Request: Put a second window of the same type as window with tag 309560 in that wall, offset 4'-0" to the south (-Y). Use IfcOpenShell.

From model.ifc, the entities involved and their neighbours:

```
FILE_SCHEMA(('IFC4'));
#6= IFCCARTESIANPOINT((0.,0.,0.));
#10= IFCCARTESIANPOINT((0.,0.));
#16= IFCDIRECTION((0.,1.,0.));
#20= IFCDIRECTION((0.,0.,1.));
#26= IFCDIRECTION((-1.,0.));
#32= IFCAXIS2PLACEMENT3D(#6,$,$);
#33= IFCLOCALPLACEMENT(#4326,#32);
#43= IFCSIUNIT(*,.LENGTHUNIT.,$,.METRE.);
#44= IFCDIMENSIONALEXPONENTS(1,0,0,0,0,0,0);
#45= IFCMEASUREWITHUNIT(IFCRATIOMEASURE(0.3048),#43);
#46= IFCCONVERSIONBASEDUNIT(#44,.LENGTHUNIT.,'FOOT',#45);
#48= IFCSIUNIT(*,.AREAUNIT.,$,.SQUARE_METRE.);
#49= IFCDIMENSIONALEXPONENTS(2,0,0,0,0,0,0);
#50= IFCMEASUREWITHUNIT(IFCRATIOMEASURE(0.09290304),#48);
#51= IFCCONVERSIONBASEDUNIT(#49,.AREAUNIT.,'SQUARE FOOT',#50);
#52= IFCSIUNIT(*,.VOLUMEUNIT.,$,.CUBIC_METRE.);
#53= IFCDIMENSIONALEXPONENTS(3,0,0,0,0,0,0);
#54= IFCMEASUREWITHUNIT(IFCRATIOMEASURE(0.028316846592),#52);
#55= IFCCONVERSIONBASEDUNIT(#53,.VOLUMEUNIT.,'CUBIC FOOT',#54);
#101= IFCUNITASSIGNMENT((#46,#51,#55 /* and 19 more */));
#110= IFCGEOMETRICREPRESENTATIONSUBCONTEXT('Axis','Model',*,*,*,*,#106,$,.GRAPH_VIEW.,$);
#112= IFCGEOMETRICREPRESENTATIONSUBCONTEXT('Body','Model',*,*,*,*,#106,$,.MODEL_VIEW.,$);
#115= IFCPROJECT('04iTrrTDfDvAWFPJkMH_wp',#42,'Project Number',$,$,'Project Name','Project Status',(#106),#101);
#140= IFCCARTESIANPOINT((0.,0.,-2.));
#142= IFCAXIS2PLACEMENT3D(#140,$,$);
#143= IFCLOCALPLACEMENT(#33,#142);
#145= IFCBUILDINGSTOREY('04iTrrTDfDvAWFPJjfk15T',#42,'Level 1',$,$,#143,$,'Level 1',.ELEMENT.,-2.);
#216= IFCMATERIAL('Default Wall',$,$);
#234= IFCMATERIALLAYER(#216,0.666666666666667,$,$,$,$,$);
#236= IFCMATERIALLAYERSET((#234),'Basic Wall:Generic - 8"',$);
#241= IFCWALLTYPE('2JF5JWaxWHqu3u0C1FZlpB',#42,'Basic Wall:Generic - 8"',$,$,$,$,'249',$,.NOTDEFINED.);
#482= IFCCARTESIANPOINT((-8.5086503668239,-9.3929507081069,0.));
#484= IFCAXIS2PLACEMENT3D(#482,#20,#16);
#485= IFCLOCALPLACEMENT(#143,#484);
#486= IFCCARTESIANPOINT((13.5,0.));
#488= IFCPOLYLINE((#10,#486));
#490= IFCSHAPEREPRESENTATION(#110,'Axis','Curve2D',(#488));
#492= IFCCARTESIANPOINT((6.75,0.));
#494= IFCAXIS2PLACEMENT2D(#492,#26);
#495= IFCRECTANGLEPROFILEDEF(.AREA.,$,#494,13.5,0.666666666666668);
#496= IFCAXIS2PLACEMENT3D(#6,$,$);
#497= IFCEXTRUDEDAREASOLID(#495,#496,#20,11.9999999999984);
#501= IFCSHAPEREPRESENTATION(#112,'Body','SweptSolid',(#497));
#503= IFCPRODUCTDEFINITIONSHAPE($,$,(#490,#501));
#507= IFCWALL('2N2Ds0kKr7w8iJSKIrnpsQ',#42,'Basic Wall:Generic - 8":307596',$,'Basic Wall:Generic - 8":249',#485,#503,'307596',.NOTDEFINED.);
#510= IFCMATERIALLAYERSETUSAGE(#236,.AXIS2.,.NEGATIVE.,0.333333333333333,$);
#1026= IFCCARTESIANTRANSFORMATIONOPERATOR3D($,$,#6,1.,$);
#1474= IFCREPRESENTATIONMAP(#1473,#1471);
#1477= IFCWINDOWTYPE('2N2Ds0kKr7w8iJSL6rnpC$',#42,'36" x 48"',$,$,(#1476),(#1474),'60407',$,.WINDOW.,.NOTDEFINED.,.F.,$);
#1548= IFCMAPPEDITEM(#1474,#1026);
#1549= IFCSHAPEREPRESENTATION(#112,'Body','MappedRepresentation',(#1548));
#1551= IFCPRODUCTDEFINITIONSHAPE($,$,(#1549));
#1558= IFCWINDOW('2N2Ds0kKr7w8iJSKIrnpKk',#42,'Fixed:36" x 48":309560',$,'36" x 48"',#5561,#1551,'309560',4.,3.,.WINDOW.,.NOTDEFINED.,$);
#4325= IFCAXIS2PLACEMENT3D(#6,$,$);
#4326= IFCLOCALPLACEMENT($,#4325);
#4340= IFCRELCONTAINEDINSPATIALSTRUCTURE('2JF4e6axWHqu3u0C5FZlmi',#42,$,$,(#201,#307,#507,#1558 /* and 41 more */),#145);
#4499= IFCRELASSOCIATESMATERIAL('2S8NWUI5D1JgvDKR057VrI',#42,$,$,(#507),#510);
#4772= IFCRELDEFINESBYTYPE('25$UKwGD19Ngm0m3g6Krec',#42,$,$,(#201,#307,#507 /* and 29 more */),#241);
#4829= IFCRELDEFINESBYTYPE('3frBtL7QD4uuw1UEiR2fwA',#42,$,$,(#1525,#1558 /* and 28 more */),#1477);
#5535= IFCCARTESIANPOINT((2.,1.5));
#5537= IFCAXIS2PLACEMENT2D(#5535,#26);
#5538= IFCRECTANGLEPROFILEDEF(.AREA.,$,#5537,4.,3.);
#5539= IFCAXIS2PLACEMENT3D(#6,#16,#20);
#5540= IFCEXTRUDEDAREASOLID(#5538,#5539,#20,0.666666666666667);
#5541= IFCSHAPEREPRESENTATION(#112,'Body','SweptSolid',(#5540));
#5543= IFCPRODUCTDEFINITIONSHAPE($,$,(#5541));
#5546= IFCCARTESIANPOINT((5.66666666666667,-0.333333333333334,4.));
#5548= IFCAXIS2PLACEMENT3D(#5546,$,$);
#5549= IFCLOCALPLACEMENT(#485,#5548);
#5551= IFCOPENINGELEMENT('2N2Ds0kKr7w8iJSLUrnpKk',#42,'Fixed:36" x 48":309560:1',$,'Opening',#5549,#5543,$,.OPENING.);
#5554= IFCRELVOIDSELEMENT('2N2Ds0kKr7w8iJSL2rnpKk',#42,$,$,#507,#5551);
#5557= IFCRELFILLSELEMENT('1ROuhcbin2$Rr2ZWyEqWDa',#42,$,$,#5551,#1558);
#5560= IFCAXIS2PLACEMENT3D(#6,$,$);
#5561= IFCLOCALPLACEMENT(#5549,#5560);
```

```python
import ifcopenshell
import ifcopenshell.api.feature
import ifcopenshell.api.geometry
import ifcopenshell.api.root
import ifcopenshell.geom
import ifcopenshell.util.element
import ifcopenshell.util.placement
import ifcopenshell.util.shape
import ifcopenshell.util.unit

model = ifcopenshell.open("model.ifc")
unit_scale = ifcopenshell.util.unit.calculate_unit_scale(model)
settings = ifcopenshell.geom.settings()


def volume(element):
    """Net volume in cubic metres, openings subtracted."""
    shape = ifcopenshell.geom.create_shape(settings, element)
    return ifcopenshell.util.shape.get_volume(shape.geometry)


def reuse_history(source, copy):
    """copy_class also copies each property set's owner history, people and application; keep the originals."""
    for rel in copy.IsDefinedBy:
        if rel.is_a("IfcRelDefinesByProperties") and (history := rel.RelatingPropertyDefinition.OwnerHistory):
            rel.RelatingPropertyDefinition.OwnerHistory = source.OwnerHistory
            ifcopenshell.util.element.remove_deep2(model, history)


window = model.by_id(1558)
opening = window.FillsVoids[0].RelatingOpeningElement
wall = opening.VoidsElements[0].RelatingBuildingElement
before = volume(wall)
shift = ifcopenshell.util.placement.get_local_placement(wall.ObjectPlacement)[:3, 0] * -48 * 0.0254 / unit_scale

# copy_class copies the void relationship, type, container and properties, but no geometry.
new_opening = ifcopenshell.api.root.copy_class(model, product=opening)
new_opening.Representation = ifcopenshell.util.element.copy_deep(
    model, opening.Representation, exclude=["IfcGeometricRepresentationContext", "IfcRepresentationMap"]
)
new_opening.Name = 'Fixed:36" x 48"'
new_window = ifcopenshell.api.root.copy_class(model, product=window)
new_window.Representation = ifcopenshell.util.element.copy_deep(
    model, window.Representation, exclude=["IfcGeometricRepresentationContext", "IfcRepresentationMap"]
)
new_window.Name = 'Fixed:36" x 48"'
new_window.Tag = None
reuse_history(window, new_window)
ifcopenshell.api.feature.add_filling(model, opening=new_opening, element=new_window)

for old, new in ((opening, new_opening), (window, new_window)):
    matrix = ifcopenshell.util.placement.get_local_placement(old.ObjectPlacement)
    matrix[:3, 3] += shift
    ifcopenshell.api.geometry.edit_object_placement(model, product=new, matrix=matrix, is_si=False)

after = volume(wall)

print(f"wall volume {before:.3f} -> {after:.3f} m3")

model.write("model-out.ifc")
```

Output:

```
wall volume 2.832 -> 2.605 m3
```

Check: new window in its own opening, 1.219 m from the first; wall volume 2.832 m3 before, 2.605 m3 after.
